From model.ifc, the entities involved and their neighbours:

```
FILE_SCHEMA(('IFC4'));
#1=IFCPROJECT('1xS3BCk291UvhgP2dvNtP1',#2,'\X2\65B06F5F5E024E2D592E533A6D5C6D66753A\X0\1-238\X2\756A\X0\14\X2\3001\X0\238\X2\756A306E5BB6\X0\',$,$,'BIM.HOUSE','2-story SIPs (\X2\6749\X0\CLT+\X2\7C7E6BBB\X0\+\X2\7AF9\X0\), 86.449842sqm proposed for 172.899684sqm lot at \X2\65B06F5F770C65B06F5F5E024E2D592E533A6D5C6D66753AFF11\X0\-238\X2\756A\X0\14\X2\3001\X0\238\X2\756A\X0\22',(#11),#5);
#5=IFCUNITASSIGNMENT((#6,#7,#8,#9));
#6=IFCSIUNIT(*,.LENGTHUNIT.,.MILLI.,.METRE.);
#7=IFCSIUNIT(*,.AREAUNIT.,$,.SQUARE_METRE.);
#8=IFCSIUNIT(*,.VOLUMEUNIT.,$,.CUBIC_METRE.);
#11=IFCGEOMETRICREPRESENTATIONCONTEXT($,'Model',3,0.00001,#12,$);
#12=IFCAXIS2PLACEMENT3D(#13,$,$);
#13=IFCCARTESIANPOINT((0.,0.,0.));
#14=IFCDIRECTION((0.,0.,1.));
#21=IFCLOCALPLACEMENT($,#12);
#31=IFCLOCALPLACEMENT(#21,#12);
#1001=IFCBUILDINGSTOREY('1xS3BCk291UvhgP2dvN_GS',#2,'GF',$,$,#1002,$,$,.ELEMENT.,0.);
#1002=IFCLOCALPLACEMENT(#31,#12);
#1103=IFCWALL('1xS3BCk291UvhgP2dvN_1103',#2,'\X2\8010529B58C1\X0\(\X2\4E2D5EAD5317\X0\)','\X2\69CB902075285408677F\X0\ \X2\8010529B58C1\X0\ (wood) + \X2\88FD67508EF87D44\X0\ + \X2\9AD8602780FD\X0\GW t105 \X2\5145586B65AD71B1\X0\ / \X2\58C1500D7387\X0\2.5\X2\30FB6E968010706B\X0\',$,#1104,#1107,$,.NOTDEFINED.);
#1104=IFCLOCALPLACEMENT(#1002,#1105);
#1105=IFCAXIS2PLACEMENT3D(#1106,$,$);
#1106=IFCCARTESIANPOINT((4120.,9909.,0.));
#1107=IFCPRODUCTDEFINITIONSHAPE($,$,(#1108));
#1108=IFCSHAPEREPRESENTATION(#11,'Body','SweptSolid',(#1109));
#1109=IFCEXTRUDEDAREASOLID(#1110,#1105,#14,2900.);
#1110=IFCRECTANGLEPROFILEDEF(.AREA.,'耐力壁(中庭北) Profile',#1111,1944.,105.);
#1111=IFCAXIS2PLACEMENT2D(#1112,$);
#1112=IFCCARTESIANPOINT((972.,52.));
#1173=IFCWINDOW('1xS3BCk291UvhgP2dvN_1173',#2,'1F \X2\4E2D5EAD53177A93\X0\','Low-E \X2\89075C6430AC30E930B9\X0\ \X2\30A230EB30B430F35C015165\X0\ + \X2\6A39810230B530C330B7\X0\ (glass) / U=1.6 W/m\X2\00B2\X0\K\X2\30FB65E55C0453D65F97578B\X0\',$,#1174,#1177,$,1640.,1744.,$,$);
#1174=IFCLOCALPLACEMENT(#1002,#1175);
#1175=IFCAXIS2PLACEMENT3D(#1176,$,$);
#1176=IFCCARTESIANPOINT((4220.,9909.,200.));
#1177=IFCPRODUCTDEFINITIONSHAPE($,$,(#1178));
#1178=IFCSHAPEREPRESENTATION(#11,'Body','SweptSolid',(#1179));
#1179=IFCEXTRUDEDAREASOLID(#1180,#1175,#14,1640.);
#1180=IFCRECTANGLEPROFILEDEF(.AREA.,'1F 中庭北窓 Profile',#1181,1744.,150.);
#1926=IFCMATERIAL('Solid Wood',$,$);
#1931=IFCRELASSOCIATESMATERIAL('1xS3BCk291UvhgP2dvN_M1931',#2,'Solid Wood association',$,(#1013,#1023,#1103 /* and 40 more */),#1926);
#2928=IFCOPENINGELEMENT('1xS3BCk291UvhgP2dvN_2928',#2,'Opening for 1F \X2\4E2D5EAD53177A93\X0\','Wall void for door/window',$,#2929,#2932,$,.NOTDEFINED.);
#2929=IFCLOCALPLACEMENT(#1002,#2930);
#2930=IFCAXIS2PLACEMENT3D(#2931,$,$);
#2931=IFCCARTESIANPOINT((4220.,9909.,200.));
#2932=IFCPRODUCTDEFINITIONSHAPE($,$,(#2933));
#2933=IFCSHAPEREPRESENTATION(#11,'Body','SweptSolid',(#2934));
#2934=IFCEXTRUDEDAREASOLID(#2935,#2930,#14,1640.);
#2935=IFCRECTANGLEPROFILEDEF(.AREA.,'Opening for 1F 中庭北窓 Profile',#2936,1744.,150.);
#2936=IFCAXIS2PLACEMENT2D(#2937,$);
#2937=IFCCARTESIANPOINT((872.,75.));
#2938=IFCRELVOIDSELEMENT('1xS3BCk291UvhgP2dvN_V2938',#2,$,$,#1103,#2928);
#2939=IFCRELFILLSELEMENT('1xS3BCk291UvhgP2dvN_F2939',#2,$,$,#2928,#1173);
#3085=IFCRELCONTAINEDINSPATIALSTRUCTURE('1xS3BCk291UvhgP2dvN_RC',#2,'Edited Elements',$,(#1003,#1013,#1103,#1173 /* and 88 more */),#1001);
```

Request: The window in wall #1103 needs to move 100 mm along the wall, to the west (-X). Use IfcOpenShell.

```python
import ifcopenshell
import ifcopenshell.api.geometry
import ifcopenshell.util.placement
import ifcopenshell.util.unit

model = ifcopenshell.open("model.ifc")
unit_scale = ifcopenshell.util.unit.calculate_unit_scale(model)

window = model.by_guid("1xS3BCk291UvhgP2dvN_1173")
opening = window.FillsVoids[0].RelatingOpeningElement
wall = opening.VoidsElements[0].RelatingBuildingElement

wall_matrix = ifcopenshell.util.placement.get_local_placement(wall.ObjectPlacement)
shift = wall_matrix[:3, 0] * -0.1 / unit_scale
before = ifcopenshell.util.placement.get_local_placement(window.ObjectPlacement)[:3, 3].copy()

# The window is not placed relative to its opening, so move both.
for product in (opening, window):
    matrix = ifcopenshell.util.placement.get_local_placement(product.ObjectPlacement)
    matrix[:3, 3] += shift
    ifcopenshell.api.geometry.edit_object_placement(model, product=product, matrix=matrix, is_si=False)

after = ifcopenshell.util.placement.get_local_placement(window.ObjectPlacement)[:3, 3]
print("window moved by", (after - before).round(3) + 0.0)

model.write("model_v2.ifc")
```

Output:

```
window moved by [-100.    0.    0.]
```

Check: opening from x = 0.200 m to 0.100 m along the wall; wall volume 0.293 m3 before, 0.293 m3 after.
